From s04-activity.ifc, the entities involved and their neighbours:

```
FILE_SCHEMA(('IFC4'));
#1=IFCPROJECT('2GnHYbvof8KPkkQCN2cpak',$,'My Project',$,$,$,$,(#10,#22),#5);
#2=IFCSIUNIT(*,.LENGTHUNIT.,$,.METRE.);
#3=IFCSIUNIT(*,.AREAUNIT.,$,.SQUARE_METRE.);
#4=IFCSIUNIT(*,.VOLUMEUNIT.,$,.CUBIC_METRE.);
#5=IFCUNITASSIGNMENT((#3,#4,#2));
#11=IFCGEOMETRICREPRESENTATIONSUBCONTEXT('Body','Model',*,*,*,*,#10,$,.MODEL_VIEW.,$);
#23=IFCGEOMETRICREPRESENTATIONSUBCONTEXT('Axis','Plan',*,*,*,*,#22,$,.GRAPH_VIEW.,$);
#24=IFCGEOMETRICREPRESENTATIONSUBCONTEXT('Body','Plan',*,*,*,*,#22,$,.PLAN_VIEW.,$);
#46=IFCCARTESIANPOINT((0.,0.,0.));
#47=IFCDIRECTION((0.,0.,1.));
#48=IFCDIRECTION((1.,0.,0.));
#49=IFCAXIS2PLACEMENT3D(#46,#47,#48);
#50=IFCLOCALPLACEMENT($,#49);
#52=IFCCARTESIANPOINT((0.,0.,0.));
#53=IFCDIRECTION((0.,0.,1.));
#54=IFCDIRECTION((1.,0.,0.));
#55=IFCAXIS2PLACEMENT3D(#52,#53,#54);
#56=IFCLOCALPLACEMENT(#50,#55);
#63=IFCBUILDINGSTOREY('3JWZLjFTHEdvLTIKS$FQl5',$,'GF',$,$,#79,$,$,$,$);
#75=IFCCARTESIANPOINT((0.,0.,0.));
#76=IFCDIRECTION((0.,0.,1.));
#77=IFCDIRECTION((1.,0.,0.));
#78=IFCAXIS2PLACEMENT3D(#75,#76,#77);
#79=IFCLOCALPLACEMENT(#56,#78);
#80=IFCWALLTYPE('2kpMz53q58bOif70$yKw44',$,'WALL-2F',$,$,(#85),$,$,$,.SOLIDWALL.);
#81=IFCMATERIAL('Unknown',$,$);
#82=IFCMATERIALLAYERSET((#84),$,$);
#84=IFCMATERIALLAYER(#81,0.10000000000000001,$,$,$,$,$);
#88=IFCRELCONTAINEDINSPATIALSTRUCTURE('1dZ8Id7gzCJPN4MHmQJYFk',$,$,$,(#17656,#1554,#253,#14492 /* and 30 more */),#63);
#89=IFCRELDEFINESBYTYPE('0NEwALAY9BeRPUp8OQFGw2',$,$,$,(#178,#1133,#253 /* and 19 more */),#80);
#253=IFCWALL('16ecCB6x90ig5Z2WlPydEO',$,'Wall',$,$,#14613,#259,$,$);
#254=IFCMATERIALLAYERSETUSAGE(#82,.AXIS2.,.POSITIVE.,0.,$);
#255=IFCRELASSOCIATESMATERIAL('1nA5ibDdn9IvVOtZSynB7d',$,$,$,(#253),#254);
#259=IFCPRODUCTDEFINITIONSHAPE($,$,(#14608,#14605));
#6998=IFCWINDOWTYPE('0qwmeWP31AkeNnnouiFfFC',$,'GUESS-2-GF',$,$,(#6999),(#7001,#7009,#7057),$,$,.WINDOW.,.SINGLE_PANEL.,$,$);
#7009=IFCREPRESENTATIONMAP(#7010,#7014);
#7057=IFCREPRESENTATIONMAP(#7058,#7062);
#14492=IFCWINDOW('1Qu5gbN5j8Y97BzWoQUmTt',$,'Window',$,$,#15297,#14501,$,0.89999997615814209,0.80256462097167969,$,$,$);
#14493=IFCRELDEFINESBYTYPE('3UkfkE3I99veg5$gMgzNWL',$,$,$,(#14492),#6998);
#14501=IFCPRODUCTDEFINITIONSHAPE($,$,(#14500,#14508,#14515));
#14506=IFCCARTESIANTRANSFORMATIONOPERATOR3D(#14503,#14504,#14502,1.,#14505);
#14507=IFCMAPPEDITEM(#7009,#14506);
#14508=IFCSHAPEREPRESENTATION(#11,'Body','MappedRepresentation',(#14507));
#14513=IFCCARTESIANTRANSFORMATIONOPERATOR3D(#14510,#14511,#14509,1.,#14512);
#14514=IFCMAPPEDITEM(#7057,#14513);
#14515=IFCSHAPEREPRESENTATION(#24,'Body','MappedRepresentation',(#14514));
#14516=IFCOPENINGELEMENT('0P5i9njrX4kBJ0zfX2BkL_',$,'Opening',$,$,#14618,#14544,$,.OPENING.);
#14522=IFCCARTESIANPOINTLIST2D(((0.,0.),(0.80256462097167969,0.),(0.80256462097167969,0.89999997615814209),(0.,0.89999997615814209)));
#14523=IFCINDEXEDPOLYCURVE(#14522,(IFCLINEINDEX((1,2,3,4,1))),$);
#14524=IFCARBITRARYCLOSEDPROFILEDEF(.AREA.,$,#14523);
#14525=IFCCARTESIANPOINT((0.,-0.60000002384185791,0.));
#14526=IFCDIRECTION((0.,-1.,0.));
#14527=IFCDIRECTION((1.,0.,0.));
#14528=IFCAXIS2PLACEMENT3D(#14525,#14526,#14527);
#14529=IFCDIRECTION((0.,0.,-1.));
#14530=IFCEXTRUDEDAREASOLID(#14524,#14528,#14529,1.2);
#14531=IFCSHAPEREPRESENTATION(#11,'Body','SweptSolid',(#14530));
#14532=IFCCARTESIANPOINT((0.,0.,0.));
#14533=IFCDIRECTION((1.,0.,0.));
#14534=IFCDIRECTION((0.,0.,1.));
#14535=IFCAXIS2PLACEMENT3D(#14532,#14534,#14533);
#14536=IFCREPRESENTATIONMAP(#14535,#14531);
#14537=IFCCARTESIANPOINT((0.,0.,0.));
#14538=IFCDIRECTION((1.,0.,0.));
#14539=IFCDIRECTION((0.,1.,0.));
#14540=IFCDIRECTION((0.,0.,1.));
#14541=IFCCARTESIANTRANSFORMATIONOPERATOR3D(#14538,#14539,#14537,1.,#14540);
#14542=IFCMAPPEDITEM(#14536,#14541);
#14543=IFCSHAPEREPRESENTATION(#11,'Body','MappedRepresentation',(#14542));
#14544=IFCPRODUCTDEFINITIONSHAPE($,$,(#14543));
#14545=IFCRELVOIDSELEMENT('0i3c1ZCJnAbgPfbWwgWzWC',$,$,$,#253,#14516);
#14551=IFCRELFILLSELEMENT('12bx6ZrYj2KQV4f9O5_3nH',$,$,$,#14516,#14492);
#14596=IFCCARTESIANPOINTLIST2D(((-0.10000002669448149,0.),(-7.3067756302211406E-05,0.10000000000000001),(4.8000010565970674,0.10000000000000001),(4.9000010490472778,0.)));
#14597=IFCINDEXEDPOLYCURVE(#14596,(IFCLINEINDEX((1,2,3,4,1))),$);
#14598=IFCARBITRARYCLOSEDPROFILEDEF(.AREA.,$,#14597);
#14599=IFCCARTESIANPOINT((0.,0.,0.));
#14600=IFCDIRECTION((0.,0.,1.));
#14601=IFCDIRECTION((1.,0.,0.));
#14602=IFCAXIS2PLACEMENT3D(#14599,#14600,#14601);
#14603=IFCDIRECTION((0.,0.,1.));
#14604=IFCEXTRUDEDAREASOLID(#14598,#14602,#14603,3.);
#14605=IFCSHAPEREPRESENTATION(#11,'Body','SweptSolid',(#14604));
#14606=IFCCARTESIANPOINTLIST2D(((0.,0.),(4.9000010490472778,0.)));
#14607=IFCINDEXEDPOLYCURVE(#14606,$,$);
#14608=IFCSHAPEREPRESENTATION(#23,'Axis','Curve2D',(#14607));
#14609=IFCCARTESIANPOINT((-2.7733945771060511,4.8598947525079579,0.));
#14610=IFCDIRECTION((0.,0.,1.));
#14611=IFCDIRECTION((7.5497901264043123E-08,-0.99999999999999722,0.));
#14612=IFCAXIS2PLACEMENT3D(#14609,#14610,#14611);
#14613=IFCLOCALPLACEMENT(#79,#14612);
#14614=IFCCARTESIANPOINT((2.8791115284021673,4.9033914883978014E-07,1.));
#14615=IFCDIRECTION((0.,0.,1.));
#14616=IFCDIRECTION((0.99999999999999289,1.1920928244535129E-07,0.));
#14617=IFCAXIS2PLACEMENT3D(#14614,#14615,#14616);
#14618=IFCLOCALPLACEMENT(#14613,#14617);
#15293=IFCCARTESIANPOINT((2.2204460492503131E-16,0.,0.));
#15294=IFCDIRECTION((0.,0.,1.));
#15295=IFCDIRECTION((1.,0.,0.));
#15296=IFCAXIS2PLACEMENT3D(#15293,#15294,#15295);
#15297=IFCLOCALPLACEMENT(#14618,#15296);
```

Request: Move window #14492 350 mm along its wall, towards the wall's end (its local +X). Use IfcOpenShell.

```python
import ifcopenshell
import ifcopenshell.api.geometry
import ifcopenshell.util.placement
import ifcopenshell.util.unit

model = ifcopenshell.open("s04-activity.ifc")
unit_scale = ifcopenshell.util.unit.calculate_unit_scale(model)

window = model.by_guid("1Qu5gbN5j8Y97BzWoQUmTt")
opening = window.FillsVoids[0].RelatingOpeningElement
wall = opening.VoidsElements[0].RelatingBuildingElement

wall_matrix = ifcopenshell.util.placement.get_local_placement(wall.ObjectPlacement)
shift = wall_matrix[:3, 0] * 0.35 / unit_scale
before = ifcopenshell.util.placement.get_local_placement(window.ObjectPlacement)[:3, 3].copy()

# The window is placed relative to its opening, so it follows when the opening moves.
matrix = ifcopenshell.util.placement.get_local_placement(opening.ObjectPlacement)
matrix[:3, 3] += shift
ifcopenshell.api.geometry.edit_object_placement(
    model, product=opening, matrix=matrix, is_si=False, should_transform_children=True
)

after = ifcopenshell.util.placement.get_local_placement(window.ObjectPlacement)[:3, 3]
print("window moved by", (after - before).round(3) + 0.0)

model.write("s04-activity_edited.ifc")
```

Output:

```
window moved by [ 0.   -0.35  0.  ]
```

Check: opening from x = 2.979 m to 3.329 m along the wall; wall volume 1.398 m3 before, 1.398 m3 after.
